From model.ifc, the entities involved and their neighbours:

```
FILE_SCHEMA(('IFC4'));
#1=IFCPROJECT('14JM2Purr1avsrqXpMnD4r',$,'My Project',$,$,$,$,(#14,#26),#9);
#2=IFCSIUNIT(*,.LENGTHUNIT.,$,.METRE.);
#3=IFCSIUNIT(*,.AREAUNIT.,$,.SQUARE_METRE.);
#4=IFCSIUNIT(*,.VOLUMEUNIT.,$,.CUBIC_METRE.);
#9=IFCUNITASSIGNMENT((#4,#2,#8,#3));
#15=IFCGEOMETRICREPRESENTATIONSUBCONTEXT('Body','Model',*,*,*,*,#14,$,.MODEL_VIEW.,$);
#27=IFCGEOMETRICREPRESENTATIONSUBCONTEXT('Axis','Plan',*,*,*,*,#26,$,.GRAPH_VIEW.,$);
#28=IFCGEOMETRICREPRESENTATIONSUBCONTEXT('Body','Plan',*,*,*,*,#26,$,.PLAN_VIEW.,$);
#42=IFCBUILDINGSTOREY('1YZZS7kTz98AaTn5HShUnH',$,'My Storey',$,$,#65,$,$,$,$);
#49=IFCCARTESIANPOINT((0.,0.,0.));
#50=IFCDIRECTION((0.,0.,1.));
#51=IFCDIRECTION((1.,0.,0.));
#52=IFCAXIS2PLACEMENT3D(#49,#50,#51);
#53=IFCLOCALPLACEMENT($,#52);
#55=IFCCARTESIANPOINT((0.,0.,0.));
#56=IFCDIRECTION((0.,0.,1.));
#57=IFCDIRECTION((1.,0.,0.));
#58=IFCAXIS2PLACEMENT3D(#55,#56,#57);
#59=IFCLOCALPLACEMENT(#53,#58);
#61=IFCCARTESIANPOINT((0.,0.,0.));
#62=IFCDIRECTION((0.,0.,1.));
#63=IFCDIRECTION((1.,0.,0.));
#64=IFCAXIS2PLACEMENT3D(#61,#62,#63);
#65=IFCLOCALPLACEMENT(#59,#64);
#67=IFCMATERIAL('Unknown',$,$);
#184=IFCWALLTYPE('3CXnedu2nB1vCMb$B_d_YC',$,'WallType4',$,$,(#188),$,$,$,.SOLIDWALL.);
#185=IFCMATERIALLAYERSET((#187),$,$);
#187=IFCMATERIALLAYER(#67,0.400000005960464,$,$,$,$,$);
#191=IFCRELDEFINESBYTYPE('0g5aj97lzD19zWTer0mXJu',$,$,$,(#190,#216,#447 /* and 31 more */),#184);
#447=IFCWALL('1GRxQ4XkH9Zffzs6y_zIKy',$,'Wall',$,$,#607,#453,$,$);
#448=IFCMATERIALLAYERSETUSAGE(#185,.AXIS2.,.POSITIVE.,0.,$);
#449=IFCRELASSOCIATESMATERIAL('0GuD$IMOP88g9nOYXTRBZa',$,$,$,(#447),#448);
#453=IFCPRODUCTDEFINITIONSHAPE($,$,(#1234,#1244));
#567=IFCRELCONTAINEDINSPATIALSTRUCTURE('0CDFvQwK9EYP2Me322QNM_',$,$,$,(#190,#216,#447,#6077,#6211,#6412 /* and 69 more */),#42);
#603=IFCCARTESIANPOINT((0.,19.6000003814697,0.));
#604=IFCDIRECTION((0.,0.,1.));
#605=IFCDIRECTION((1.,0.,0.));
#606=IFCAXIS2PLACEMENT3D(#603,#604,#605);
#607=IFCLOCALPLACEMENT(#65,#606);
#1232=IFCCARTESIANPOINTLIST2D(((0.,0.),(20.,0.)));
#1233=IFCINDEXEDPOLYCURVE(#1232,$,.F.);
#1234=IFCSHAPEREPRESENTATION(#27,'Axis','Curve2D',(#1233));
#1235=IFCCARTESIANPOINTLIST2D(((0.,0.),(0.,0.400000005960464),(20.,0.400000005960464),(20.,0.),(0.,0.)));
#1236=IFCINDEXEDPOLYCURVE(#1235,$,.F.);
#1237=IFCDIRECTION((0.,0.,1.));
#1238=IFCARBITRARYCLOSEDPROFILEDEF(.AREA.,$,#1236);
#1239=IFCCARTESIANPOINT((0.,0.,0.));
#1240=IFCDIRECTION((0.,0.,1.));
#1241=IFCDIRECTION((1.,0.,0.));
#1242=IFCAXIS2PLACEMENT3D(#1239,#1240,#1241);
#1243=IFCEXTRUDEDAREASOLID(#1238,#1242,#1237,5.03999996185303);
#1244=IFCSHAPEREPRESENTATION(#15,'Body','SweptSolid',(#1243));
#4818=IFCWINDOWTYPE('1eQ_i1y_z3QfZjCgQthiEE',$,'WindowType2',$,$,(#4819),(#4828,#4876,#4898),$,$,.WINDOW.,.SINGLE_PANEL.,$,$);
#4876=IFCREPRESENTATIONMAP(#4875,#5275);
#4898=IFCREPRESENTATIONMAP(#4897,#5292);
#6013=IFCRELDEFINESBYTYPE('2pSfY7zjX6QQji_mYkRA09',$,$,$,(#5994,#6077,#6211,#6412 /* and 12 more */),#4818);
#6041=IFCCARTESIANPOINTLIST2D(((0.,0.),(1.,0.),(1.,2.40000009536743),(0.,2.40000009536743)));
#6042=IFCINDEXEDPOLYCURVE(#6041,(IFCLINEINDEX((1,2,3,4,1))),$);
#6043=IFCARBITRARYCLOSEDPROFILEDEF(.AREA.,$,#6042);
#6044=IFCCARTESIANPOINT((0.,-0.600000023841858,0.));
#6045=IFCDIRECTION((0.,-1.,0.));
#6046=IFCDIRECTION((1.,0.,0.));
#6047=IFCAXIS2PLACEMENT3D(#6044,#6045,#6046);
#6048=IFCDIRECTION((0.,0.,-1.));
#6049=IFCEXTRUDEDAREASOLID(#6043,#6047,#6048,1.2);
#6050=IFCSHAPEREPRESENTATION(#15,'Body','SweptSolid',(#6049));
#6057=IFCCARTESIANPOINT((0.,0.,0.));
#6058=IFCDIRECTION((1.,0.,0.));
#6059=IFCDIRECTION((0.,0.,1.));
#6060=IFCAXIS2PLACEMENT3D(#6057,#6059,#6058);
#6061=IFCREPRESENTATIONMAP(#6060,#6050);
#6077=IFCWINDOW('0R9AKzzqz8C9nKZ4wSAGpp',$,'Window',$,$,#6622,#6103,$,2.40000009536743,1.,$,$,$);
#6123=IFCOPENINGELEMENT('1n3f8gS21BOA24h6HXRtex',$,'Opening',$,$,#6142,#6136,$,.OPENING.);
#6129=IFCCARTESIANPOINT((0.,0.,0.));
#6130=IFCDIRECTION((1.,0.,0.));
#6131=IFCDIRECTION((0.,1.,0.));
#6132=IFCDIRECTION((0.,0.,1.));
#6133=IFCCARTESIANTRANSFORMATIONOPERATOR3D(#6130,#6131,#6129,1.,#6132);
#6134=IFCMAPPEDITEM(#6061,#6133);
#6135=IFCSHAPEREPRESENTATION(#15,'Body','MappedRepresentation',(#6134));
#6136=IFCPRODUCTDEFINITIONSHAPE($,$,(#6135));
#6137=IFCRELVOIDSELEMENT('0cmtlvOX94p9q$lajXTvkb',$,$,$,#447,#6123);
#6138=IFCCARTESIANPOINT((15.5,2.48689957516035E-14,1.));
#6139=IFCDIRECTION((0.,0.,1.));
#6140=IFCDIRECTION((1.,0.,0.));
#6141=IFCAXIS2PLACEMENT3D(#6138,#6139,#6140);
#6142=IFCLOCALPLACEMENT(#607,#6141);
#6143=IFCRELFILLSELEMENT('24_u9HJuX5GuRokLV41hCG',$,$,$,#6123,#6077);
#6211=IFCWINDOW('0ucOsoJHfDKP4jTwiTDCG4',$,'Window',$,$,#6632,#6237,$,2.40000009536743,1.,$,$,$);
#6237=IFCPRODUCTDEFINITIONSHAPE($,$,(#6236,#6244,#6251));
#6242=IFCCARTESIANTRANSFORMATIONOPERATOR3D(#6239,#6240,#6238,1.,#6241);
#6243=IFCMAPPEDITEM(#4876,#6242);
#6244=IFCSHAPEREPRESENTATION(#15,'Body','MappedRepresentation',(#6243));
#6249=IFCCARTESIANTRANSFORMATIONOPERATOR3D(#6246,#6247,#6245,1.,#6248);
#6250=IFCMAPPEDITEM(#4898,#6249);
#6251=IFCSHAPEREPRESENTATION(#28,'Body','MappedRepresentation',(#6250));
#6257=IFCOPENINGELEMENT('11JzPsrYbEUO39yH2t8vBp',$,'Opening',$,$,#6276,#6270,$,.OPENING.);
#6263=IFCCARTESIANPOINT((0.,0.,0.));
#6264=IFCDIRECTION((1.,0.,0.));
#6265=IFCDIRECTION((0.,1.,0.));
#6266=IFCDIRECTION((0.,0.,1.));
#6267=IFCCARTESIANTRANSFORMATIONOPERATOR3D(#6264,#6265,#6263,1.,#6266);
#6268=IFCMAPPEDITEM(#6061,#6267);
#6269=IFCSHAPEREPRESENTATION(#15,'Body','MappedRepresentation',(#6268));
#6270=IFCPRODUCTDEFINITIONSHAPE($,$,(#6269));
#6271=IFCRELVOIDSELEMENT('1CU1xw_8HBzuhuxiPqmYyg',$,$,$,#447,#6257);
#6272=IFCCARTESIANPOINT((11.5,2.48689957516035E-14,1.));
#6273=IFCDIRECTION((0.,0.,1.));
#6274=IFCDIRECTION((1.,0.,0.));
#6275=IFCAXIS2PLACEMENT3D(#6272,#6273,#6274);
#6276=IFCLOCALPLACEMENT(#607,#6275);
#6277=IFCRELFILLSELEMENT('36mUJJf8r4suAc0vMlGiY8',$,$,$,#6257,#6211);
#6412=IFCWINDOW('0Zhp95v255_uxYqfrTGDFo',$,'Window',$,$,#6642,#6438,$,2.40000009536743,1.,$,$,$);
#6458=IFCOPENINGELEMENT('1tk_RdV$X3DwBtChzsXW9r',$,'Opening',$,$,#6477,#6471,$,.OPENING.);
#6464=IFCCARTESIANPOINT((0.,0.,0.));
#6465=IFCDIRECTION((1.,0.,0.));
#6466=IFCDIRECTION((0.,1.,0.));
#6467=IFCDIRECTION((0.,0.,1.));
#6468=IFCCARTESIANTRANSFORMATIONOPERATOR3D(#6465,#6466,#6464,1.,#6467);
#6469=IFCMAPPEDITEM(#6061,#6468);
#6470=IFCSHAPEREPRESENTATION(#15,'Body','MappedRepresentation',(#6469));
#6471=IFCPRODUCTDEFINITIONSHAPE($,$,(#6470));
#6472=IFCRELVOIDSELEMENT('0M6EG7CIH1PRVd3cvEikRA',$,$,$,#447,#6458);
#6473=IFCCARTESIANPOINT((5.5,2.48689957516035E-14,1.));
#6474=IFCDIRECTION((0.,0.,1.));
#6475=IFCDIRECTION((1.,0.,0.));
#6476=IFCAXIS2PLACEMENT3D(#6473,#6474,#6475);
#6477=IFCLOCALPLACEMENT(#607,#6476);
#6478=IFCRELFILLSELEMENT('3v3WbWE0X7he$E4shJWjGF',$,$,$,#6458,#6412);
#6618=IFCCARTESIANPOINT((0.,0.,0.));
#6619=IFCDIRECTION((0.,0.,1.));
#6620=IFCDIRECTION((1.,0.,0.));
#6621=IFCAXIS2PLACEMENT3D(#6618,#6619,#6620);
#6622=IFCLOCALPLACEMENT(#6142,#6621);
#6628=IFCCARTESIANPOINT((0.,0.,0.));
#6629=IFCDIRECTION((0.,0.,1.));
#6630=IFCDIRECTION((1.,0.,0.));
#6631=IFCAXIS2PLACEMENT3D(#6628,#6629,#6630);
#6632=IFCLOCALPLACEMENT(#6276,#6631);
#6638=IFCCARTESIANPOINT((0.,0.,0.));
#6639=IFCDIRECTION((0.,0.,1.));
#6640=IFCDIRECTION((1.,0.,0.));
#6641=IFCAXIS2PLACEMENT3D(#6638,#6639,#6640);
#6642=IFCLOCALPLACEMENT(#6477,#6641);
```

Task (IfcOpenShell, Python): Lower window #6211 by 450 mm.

```python
import numpy as np
import ifcopenshell
import ifcopenshell.api.geometry
import ifcopenshell.util.placement
import ifcopenshell.util.unit

model = ifcopenshell.open("model.ifc")
unit_scale = ifcopenshell.util.unit.calculate_unit_scale(model)

window = model.by_guid("0ucOsoJHfDKP4jTwiTDCG4")
opening = window.FillsVoids[0].RelatingOpeningElement
dz = -0.45 / unit_scale

shift = np.array([0.0, 0.0, dz])
# The window is placed relative to its opening, so it follows when the opening moves.
matrix = ifcopenshell.util.placement.get_local_placement(opening.ObjectPlacement)
matrix[:3, 3] += shift
ifcopenshell.api.geometry.edit_object_placement(
    model, product=opening, matrix=matrix, is_si=False, should_transform_children=True
)

print(f"moved by {dz * unit_scale:+.3f} m")

model.write("model_rev.ifc")
```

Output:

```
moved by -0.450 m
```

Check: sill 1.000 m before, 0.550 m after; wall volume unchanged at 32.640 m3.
